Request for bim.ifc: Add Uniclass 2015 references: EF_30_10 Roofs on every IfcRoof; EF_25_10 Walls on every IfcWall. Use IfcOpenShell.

First a look at what the model holds.

```python
import ifcopenshell

model = ifcopenshell.open("bim.ifc")
print(model.schema)
print("classifications:", [c.Name for c in model.by_type("IfcClassification")])
for ifc_class in ("IfcDoor", "IfcRoof", "IfcStair", "IfcWall", "IfcWindow"):
    print(ifc_class, len(model.by_type(ifc_class)))
```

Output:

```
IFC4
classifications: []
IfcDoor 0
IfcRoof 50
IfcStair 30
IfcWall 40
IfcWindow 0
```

```python
import ifcopenshell
import ifcopenshell.api.classification

model = ifcopenshell.open("bim.ifc")

system = ifcopenshell.api.classification.add_classification(model, classification="Uniclass 2015")

codes = {
    "IfcRoof": ("EF_30_10", "Roofs"),
    "IfcWall": ("EF_25_10", "Walls"),
}
for ifc_class, (code, name) in codes.items():
    products = model.by_type(ifc_class)
    ifcopenshell.api.classification.add_reference(
        model, products=products, classification=system, identification=code, name=name
    )
    print(code, len(products))

model.write("bim_updated.ifc")
```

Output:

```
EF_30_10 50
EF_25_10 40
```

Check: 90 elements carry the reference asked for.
